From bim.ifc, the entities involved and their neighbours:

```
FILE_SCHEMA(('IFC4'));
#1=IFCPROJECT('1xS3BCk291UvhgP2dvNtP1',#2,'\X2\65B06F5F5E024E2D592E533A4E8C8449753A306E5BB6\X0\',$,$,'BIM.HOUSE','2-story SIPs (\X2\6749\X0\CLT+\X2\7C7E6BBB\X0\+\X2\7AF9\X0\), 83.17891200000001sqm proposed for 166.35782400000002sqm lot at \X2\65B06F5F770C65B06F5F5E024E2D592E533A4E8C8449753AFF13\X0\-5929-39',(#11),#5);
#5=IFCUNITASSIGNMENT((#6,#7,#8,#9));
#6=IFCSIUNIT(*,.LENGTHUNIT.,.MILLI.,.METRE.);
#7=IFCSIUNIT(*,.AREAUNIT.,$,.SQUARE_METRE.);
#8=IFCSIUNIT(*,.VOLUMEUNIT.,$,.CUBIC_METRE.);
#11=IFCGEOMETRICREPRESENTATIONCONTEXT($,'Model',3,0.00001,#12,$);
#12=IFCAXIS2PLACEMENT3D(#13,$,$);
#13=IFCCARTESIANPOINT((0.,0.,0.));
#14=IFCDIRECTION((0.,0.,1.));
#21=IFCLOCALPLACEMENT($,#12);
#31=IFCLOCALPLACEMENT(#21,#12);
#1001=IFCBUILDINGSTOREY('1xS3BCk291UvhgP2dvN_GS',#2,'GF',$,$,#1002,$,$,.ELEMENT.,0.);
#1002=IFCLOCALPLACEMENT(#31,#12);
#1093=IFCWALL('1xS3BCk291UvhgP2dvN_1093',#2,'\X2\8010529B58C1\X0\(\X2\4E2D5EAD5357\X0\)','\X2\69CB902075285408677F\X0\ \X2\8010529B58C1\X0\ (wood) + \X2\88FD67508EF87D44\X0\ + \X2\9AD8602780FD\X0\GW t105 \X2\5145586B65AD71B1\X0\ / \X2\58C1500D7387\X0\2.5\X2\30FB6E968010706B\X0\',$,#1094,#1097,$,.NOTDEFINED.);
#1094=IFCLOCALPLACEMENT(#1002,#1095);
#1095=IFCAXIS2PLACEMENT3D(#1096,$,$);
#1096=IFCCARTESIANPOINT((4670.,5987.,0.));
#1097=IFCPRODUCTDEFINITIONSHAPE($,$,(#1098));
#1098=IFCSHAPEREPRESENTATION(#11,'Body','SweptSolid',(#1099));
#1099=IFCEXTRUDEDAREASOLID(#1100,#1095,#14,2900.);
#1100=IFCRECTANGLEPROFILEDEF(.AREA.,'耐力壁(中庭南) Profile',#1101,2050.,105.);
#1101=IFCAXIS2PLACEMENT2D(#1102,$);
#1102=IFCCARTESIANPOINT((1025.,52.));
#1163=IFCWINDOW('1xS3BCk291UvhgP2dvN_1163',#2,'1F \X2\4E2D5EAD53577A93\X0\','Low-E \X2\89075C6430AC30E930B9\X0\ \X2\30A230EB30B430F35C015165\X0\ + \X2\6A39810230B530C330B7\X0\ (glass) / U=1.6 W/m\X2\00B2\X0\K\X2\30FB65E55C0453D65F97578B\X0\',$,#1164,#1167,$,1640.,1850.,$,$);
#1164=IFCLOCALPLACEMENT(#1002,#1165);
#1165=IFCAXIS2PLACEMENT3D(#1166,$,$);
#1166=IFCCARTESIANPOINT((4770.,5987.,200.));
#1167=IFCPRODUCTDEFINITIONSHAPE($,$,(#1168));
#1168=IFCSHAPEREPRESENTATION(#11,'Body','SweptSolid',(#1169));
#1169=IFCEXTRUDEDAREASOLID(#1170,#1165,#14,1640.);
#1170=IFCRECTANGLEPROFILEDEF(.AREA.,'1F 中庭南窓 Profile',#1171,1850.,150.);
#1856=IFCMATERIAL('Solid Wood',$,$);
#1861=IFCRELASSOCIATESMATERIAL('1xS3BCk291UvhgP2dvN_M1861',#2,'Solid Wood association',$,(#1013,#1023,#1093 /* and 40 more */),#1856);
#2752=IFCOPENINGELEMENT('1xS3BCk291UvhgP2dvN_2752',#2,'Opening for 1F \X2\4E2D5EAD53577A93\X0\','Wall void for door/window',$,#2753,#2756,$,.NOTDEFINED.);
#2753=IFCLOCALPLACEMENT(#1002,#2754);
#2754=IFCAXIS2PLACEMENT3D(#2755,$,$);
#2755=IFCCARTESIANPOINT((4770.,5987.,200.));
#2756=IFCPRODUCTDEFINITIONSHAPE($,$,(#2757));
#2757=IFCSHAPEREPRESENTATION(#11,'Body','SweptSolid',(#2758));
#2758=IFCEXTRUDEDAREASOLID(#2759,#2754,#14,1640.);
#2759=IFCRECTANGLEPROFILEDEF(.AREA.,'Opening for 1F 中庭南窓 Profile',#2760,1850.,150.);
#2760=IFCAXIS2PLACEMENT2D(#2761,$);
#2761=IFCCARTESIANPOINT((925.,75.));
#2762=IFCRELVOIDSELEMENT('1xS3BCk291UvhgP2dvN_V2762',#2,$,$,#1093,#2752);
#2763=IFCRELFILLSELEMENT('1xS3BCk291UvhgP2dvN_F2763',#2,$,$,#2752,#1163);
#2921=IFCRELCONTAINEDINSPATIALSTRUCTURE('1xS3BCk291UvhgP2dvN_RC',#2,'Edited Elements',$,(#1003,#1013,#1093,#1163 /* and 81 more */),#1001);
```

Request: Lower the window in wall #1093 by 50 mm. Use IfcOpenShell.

```python
import numpy as np
import ifcopenshell
import ifcopenshell.api.geometry
import ifcopenshell.util.placement
import ifcopenshell.util.unit

model = ifcopenshell.open("bim.ifc")
unit_scale = ifcopenshell.util.unit.calculate_unit_scale(model)

window = model.by_id(1163)
opening = window.FillsVoids[0].RelatingOpeningElement
dz = -0.05 / unit_scale

shift = np.array([0.0, 0.0, dz])
# The window is not placed relative to its opening, so move both.
for product in (opening, window):
    matrix = ifcopenshell.util.placement.get_local_placement(product.ObjectPlacement)
    matrix[:3, 3] += shift
    ifcopenshell.api.geometry.edit_object_placement(model, product=product, matrix=matrix, is_si=False)

print(f"moved by {dz * unit_scale:+.3f} m")

model.write("bim_updated.ifc")
```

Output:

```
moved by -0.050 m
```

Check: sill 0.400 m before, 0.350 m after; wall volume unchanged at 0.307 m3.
